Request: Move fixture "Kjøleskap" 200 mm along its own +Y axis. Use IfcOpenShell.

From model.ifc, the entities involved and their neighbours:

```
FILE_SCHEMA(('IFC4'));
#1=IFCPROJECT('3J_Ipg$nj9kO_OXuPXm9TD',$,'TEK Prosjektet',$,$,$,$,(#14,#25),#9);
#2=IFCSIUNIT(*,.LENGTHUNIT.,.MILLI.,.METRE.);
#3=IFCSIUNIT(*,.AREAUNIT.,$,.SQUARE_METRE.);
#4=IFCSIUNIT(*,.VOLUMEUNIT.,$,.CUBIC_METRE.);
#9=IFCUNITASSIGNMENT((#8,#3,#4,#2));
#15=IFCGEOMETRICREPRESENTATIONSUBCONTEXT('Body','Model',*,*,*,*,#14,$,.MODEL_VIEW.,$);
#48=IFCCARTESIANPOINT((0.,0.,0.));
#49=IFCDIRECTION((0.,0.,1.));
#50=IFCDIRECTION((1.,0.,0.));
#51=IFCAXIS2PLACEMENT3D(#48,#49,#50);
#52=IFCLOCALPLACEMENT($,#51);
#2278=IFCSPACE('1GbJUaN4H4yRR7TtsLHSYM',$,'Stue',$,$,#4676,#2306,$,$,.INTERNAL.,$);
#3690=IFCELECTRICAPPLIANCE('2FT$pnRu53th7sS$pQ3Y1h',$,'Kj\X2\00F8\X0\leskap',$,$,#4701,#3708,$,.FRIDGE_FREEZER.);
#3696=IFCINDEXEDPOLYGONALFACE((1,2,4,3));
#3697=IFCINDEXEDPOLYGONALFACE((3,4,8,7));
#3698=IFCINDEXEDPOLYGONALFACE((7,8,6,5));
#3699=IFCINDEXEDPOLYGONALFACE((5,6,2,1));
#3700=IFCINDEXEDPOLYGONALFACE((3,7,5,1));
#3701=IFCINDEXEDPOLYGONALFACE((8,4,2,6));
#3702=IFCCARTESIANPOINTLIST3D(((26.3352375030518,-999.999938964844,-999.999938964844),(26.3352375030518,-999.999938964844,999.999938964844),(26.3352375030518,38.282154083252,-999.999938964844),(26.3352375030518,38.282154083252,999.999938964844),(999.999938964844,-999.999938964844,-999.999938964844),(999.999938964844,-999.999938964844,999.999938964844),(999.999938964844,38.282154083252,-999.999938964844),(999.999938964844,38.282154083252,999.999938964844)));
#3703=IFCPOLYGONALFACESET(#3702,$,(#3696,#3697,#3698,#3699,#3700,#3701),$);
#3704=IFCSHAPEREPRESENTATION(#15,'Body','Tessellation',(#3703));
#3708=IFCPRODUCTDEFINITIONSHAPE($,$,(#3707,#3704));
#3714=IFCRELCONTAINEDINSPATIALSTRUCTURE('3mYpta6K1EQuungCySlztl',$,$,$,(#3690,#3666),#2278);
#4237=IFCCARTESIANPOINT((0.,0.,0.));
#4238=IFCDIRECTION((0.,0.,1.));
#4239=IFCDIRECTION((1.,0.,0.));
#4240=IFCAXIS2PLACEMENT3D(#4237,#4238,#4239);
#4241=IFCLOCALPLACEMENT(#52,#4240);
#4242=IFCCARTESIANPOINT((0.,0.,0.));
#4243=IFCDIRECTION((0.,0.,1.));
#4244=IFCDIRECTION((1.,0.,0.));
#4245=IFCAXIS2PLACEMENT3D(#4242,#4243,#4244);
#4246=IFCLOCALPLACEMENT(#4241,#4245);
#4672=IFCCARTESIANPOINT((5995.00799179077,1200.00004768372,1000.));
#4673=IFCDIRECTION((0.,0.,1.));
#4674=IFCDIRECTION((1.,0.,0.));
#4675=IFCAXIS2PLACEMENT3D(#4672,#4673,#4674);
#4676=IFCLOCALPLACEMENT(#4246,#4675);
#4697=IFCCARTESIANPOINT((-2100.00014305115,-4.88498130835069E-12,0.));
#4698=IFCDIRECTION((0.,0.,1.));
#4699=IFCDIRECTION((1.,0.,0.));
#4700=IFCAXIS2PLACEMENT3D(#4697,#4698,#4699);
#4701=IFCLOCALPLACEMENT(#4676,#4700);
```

```python
import ifcopenshell
import ifcopenshell.api.geometry
import ifcopenshell.util.placement

model = ifcopenshell.open("model.ifc")

item = model.by_guid("2FT$pnRu53th7sS$pQ3Y1h")
matrix = ifcopenshell.util.placement.get_local_placement(item.ObjectPlacement)
matrix[:3, 3] += matrix[:3, 1] * 200.0
ifcopenshell.api.geometry.edit_object_placement(model, product=item, matrix=matrix, is_si=False)

print(ifcopenshell.util.placement.get_local_placement(item.ObjectPlacement).round(3) + 0.0)

model.write("model-out.ifc")
```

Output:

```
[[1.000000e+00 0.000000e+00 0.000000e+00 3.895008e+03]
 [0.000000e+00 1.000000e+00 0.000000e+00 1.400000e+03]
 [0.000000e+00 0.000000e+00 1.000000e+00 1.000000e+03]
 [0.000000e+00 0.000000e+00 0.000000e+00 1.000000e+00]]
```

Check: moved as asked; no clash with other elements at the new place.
